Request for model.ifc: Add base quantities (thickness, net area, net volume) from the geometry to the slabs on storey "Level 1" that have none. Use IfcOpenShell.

First a look at what the model holds.

```python
import ifcopenshell
import ifcopenshell.util.element
import ifcopenshell.util.unit

model = ifcopenshell.open("model.ifc")
print(model.schema)
for unit_type in ("LENGTHUNIT", "AREAUNIT", "VOLUMEUNIT"):
    print(unit_type, ifcopenshell.util.unit.calculate_unit_scale(model, unit_type))
storey = next(s for s in model.by_type("IfcBuildingStorey") if s.Name == "Level 1")
slabs = [e for e in ifcopenshell.util.element.get_decomposition(storey) if e.is_a("IfcSlab")]
for e in sorted(slabs, key=lambda e: e.id()):
    print(e.id(), e.is_a(), e.Name, list(ifcopenshell.util.element.get_psets(e, qtos_only=True)), sep=" | ")
```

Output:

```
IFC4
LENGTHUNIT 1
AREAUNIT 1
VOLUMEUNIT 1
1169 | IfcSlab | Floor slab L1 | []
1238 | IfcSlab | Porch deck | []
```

```python
import ifcopenshell
import ifcopenshell.api.pset
import ifcopenshell.geom
import ifcopenshell.util.element
import ifcopenshell.util.shape
import ifcopenshell.util.unit

model = ifcopenshell.open("model.ifc")
unit_scale = ifcopenshell.util.unit.calculate_unit_scale(model)
area_scale = ifcopenshell.util.unit.calculate_unit_scale(model, "AREAUNIT")
volume_scale = ifcopenshell.util.unit.calculate_unit_scale(model, "VOLUMEUNIT")
settings = ifcopenshell.geom.settings()

storey = next(s for s in model.by_type("IfcBuildingStorey") if s.Name == "Level 1")
slabs = [e for e in ifcopenshell.util.element.get_decomposition(storey) if e.is_a("IfcSlab")]

for e in sorted(slabs, key=lambda e: e.id()):
    if ifcopenshell.util.element.get_psets(e, qtos_only=True, should_inherit=False):
        continue
    # Geometry comes back in metres, in the element's own axes.
    shape = ifcopenshell.geom.create_shape(settings, e)
    values = {
        "Width": ifcopenshell.util.shape.get_z(shape.geometry) / unit_scale,
        "NetArea": ifcopenshell.util.shape.get_footprint_area(shape.geometry) / area_scale,
        "NetVolume": ifcopenshell.util.shape.get_volume(shape.geometry) / volume_scale,
    }
    qto = ifcopenshell.api.pset.add_qto(model, product=e, name="Qto_SlabBaseQuantities")
    ifcopenshell.api.pset.edit_qto(model, qto=qto, properties=values)
    print(e.id(), {k: round(v, 3) for k, v in values.items()})

model.write("model_v2.ifc")
```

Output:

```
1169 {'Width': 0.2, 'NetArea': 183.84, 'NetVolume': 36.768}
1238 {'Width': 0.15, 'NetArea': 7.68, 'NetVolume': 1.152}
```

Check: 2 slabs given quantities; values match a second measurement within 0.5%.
